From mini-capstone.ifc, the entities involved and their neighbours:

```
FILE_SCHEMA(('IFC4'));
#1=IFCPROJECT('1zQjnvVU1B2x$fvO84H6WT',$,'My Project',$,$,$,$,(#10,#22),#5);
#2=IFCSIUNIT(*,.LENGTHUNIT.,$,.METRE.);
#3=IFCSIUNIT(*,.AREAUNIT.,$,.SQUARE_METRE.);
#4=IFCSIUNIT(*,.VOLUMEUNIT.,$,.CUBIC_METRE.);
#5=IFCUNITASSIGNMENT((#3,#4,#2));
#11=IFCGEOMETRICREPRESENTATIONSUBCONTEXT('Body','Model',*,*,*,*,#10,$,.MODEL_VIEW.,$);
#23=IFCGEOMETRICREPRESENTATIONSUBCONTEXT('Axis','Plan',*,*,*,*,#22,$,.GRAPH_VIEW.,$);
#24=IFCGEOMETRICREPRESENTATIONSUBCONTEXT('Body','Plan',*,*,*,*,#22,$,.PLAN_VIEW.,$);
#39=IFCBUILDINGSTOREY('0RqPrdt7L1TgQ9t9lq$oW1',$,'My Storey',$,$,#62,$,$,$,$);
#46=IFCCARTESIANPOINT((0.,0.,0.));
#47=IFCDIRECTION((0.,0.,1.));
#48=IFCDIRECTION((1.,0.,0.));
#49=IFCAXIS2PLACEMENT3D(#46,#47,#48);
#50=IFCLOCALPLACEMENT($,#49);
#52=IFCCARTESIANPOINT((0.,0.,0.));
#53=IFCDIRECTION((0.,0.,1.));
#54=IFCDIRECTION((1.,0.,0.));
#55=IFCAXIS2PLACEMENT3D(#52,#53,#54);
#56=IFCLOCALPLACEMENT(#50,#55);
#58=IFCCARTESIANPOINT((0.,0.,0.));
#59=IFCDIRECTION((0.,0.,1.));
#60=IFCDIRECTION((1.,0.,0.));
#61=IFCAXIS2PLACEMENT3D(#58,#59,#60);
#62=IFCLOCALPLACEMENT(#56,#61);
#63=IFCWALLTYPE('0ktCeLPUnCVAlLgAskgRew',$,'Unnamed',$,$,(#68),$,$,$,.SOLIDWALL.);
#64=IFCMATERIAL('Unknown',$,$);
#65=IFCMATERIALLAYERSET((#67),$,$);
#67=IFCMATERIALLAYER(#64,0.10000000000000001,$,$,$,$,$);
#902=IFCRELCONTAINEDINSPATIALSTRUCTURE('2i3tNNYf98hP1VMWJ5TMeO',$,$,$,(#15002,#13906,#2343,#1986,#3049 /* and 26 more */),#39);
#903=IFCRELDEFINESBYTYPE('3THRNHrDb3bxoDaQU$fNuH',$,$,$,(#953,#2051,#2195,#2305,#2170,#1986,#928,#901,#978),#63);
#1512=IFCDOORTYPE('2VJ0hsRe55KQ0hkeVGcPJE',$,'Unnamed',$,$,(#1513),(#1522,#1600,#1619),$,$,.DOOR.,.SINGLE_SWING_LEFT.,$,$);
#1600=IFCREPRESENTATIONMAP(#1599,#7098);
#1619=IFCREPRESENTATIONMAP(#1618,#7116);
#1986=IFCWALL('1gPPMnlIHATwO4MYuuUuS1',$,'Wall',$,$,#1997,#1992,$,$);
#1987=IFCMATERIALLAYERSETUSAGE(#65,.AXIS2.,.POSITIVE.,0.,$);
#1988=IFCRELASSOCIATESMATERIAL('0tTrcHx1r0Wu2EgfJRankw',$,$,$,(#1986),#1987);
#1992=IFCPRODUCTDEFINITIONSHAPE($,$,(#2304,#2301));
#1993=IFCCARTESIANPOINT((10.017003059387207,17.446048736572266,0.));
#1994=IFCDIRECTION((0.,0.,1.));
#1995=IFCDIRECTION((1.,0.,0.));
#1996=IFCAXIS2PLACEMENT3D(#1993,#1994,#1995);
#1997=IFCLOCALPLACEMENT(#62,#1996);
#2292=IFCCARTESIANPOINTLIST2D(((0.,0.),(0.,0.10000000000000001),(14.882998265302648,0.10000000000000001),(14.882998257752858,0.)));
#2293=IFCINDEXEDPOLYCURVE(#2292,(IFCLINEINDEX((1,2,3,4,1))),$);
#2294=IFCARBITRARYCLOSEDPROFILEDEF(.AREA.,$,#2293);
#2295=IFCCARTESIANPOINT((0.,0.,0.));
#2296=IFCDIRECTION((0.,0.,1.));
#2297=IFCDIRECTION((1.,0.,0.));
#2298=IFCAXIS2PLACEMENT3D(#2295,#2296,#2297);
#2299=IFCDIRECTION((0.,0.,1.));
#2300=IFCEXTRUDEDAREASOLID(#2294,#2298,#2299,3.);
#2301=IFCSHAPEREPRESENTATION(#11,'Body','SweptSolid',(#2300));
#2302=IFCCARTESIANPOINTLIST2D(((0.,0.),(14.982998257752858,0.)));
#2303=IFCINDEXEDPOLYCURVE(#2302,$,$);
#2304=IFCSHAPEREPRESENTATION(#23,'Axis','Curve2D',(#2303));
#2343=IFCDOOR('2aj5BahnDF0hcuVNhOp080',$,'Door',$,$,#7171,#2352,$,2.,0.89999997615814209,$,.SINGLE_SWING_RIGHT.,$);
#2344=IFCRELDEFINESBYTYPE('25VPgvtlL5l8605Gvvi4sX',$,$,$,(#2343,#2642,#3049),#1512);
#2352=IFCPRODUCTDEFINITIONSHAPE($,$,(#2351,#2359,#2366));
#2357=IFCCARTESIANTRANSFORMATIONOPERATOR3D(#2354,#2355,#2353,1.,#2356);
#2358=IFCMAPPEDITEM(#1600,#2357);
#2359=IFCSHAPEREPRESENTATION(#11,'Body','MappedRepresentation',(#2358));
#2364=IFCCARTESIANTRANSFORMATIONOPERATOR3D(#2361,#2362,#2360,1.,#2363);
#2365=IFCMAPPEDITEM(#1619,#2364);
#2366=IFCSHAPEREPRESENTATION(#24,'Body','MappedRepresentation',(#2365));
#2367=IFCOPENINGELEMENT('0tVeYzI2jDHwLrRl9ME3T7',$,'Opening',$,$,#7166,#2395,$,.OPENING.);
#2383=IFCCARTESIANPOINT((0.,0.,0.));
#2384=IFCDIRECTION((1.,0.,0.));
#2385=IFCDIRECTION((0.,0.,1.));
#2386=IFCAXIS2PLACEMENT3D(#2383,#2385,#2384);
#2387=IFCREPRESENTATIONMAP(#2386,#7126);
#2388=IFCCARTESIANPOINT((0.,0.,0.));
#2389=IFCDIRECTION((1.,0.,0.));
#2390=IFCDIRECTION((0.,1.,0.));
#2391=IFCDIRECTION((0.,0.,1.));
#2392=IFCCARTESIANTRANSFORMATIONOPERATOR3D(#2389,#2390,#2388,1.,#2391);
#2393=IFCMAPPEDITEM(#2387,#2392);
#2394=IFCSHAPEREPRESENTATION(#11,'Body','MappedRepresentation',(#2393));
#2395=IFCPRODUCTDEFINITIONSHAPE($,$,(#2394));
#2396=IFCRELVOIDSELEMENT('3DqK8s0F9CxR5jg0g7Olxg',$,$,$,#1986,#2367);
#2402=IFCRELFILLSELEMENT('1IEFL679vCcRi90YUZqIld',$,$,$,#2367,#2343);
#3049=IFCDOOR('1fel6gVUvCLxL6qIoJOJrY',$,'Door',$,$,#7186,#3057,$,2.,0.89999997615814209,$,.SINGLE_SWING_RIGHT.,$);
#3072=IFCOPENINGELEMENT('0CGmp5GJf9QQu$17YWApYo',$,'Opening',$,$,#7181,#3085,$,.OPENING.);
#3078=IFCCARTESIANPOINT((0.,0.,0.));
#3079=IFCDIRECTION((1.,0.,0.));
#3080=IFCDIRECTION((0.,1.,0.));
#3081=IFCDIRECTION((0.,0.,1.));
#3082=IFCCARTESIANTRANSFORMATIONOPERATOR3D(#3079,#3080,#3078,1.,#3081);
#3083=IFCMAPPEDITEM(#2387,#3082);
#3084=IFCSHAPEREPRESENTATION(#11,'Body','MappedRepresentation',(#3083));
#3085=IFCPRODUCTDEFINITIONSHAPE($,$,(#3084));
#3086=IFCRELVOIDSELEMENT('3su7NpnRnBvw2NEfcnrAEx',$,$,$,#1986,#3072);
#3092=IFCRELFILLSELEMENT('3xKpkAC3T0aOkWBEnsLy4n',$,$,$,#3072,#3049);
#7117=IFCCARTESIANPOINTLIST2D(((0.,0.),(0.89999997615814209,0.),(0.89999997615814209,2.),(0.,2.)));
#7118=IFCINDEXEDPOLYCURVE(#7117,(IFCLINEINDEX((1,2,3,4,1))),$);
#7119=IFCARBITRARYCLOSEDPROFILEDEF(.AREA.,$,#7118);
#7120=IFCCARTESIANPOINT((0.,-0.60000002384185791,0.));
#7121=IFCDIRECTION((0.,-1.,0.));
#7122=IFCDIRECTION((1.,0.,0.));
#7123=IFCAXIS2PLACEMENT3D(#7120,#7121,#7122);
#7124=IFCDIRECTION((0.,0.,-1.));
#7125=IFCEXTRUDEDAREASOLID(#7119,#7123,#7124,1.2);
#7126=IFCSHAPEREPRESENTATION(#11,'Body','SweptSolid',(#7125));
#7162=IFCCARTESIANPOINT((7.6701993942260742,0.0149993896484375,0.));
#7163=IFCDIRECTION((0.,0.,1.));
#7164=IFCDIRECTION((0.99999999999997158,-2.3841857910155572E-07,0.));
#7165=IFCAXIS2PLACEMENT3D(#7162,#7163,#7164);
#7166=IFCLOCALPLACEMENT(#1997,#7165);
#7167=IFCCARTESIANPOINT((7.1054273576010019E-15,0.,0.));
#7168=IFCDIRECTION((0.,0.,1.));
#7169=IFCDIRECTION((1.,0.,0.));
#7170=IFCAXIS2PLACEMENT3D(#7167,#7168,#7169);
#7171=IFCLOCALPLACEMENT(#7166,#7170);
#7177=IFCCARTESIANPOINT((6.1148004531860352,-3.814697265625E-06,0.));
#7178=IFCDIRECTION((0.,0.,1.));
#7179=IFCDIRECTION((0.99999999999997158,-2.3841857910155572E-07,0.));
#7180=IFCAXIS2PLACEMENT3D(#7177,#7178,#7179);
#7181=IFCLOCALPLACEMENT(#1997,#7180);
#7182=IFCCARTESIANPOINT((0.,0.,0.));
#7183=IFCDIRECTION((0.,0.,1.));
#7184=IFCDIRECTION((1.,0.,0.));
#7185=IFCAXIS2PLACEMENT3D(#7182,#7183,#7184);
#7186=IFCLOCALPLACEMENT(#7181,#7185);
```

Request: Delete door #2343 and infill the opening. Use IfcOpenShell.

```python
import ifcopenshell
import ifcopenshell.api.feature
import ifcopenshell.api.root
import ifcopenshell.geom
import ifcopenshell.util.shape

model = ifcopenshell.open("mini-capstone.ifc")
settings = ifcopenshell.geom.settings()


def volume(element):
    """Net volume in cubic metres, openings subtracted."""
    shape = ifcopenshell.geom.create_shape(settings, element)
    return ifcopenshell.util.shape.get_volume(shape.geometry)


door = model.by_id(2343)
opening = door.FillsVoids[0].RelatingOpeningElement
wall = opening.VoidsElements[0].RelatingBuildingElement
before = volume(wall)

ifcopenshell.api.root.remove_product(model, product=door)
ifcopenshell.api.feature.remove_feature(model, feature=opening)

after = volume(wall)

print(f"wall volume {before:.3f} -> {after:.3f} m3")

model.write("mini-capstone_updated.ifc")
```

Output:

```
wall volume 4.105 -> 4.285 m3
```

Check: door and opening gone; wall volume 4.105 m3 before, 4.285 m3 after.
